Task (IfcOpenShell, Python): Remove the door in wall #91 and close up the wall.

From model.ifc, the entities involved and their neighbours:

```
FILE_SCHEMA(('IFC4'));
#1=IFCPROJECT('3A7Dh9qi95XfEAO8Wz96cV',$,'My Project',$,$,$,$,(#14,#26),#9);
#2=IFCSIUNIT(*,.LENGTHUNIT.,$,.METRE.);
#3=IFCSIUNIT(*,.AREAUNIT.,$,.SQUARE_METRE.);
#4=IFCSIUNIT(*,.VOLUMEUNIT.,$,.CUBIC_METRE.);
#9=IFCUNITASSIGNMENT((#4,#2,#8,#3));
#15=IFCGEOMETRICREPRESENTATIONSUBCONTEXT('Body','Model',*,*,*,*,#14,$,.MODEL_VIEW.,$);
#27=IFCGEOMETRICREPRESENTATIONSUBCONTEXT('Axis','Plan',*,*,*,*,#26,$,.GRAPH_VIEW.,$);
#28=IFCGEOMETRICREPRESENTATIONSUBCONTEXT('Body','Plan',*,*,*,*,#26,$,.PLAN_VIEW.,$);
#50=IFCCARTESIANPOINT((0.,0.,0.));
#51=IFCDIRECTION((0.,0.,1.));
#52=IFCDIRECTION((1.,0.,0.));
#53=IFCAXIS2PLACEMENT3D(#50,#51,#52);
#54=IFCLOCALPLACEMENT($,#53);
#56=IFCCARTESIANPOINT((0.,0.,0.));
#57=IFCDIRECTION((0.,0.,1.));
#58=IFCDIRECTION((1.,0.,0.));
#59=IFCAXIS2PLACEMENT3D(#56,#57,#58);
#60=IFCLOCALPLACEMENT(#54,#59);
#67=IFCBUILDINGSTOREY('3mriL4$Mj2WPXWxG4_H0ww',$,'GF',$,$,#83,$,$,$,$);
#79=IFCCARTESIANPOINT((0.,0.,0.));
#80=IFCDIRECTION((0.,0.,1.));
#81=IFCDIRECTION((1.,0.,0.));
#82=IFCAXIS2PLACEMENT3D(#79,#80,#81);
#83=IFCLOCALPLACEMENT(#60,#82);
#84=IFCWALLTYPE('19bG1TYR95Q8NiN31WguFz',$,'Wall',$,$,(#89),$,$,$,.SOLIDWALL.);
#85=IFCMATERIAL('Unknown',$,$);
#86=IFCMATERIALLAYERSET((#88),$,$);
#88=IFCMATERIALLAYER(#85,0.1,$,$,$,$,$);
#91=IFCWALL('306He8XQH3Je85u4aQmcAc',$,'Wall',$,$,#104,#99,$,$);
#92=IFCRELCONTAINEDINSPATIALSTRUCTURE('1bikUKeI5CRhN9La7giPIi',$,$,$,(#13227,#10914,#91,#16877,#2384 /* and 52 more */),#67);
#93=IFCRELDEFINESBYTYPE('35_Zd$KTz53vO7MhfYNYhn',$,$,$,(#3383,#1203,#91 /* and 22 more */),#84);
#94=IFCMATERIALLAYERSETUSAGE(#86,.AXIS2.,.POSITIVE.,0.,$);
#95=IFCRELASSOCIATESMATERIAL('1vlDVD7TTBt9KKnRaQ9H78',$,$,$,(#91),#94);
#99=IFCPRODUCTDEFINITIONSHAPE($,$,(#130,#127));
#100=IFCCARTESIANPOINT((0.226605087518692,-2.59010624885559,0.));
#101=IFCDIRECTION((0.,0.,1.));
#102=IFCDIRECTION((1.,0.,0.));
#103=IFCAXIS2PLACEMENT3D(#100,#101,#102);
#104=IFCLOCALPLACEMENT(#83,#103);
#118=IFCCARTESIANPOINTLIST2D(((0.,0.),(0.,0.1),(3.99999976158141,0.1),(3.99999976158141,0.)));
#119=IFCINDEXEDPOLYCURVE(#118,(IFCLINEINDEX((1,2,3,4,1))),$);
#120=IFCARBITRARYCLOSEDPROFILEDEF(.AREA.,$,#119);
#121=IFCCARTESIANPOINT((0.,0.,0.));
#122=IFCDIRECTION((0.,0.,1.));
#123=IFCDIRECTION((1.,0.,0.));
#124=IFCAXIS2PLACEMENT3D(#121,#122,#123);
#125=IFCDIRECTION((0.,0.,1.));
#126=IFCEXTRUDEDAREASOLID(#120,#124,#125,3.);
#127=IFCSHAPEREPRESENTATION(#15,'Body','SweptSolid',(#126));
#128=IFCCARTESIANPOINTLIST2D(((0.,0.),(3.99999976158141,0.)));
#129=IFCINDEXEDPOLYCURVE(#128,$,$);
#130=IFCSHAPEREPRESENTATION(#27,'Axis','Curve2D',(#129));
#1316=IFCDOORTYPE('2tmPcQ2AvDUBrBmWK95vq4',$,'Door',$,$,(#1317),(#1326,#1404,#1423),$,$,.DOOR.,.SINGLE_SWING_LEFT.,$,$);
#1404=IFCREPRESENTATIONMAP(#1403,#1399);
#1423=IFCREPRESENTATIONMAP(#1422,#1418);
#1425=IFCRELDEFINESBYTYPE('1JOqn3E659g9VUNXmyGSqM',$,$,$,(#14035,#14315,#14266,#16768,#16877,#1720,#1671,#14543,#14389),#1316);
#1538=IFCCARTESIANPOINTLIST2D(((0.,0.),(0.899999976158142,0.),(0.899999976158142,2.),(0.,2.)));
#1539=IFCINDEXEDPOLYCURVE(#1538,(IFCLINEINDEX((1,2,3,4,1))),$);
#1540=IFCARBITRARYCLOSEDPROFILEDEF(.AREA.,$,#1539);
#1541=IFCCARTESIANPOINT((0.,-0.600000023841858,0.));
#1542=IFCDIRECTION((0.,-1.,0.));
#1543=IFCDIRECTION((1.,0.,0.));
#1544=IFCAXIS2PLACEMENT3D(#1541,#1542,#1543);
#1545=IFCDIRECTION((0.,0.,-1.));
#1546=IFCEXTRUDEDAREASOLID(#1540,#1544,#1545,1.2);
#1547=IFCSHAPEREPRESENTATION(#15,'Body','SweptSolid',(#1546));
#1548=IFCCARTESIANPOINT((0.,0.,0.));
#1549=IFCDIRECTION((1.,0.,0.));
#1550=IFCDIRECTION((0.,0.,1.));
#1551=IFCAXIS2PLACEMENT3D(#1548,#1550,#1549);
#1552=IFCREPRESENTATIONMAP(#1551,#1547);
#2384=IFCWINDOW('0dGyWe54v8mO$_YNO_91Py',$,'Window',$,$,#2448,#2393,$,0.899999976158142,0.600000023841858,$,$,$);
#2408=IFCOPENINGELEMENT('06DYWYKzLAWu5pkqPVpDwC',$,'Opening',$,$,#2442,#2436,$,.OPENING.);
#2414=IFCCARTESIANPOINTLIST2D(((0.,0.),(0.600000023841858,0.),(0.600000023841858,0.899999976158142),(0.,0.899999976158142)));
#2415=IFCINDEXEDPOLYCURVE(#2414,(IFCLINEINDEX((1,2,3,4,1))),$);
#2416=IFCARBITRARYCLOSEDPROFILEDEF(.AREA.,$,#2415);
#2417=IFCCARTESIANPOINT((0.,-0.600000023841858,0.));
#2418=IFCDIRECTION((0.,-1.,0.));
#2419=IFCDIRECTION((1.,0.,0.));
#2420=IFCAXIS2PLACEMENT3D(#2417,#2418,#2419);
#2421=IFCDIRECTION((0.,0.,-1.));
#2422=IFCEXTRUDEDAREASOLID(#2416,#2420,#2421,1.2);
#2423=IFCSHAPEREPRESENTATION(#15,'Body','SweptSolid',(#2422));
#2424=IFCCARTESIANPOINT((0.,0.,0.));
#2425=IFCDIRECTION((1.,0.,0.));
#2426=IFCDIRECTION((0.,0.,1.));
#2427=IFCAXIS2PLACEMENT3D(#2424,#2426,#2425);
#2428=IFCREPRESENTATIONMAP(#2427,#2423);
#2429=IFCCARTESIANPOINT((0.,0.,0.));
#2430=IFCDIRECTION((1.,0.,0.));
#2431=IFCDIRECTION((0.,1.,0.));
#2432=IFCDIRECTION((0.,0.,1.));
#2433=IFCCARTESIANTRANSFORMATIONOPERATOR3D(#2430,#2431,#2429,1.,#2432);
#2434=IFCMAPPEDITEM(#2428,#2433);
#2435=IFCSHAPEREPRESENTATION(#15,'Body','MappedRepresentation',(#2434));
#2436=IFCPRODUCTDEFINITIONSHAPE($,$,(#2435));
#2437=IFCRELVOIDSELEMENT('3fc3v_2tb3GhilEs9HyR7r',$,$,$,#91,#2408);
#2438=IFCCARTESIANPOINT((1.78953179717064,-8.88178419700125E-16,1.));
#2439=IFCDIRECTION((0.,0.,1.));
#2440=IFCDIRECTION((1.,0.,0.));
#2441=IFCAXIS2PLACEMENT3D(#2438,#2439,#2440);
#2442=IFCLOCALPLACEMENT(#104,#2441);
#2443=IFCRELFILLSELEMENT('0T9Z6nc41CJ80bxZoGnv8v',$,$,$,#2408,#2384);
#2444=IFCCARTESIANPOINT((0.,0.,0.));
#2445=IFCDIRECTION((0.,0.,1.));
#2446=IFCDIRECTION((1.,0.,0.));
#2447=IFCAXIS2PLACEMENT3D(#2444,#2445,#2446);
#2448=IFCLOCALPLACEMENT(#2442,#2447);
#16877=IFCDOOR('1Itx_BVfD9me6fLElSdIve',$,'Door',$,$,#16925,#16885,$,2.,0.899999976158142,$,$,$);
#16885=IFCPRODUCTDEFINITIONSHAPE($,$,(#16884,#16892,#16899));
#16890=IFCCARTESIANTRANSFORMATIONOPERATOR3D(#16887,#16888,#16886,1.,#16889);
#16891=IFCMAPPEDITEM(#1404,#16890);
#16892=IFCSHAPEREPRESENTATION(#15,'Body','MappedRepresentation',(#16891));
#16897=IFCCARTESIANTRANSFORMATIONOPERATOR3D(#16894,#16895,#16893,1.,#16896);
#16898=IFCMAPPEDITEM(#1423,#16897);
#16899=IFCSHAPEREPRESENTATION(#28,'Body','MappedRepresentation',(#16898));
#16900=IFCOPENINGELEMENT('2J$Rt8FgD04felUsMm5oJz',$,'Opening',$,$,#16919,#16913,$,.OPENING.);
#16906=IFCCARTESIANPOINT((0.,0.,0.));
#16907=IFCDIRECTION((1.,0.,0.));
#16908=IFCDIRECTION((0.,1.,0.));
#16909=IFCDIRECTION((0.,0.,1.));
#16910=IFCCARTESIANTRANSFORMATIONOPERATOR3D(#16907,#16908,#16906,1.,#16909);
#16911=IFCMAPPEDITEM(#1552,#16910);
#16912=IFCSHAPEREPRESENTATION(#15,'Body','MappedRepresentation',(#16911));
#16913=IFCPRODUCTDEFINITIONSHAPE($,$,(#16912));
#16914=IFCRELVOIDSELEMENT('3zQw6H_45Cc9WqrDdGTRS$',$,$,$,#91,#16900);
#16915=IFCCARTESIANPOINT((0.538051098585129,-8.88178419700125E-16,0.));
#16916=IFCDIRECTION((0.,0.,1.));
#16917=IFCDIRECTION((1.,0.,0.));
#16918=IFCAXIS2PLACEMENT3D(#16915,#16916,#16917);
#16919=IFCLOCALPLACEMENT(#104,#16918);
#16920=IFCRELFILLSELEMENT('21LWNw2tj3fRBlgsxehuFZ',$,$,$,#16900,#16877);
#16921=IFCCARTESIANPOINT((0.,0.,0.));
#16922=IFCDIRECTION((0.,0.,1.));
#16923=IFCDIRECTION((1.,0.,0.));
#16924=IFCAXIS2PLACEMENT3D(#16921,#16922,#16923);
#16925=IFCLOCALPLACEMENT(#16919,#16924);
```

```python
import ifcopenshell
import ifcopenshell.api.feature
import ifcopenshell.api.root
import ifcopenshell.geom
import ifcopenshell.util.shape

model = ifcopenshell.open("model.ifc")
settings = ifcopenshell.geom.settings()


def volume(element):
    """Net volume in cubic metres, openings subtracted."""
    shape = ifcopenshell.geom.create_shape(settings, element)
    return ifcopenshell.util.shape.get_volume(shape.geometry)


door = model.by_guid("1Itx_BVfD9me6fLElSdIve")
opening = door.FillsVoids[0].RelatingOpeningElement
wall = opening.VoidsElements[0].RelatingBuildingElement
before = volume(wall)

ifcopenshell.api.root.remove_product(model, product=door)
ifcopenshell.api.feature.remove_feature(model, feature=opening)

after = volume(wall)

print(f"wall volume {before:.3f} -> {after:.3f} m3")

model.write("model_edited.ifc")
```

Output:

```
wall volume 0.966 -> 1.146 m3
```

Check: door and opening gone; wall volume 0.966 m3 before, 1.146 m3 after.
